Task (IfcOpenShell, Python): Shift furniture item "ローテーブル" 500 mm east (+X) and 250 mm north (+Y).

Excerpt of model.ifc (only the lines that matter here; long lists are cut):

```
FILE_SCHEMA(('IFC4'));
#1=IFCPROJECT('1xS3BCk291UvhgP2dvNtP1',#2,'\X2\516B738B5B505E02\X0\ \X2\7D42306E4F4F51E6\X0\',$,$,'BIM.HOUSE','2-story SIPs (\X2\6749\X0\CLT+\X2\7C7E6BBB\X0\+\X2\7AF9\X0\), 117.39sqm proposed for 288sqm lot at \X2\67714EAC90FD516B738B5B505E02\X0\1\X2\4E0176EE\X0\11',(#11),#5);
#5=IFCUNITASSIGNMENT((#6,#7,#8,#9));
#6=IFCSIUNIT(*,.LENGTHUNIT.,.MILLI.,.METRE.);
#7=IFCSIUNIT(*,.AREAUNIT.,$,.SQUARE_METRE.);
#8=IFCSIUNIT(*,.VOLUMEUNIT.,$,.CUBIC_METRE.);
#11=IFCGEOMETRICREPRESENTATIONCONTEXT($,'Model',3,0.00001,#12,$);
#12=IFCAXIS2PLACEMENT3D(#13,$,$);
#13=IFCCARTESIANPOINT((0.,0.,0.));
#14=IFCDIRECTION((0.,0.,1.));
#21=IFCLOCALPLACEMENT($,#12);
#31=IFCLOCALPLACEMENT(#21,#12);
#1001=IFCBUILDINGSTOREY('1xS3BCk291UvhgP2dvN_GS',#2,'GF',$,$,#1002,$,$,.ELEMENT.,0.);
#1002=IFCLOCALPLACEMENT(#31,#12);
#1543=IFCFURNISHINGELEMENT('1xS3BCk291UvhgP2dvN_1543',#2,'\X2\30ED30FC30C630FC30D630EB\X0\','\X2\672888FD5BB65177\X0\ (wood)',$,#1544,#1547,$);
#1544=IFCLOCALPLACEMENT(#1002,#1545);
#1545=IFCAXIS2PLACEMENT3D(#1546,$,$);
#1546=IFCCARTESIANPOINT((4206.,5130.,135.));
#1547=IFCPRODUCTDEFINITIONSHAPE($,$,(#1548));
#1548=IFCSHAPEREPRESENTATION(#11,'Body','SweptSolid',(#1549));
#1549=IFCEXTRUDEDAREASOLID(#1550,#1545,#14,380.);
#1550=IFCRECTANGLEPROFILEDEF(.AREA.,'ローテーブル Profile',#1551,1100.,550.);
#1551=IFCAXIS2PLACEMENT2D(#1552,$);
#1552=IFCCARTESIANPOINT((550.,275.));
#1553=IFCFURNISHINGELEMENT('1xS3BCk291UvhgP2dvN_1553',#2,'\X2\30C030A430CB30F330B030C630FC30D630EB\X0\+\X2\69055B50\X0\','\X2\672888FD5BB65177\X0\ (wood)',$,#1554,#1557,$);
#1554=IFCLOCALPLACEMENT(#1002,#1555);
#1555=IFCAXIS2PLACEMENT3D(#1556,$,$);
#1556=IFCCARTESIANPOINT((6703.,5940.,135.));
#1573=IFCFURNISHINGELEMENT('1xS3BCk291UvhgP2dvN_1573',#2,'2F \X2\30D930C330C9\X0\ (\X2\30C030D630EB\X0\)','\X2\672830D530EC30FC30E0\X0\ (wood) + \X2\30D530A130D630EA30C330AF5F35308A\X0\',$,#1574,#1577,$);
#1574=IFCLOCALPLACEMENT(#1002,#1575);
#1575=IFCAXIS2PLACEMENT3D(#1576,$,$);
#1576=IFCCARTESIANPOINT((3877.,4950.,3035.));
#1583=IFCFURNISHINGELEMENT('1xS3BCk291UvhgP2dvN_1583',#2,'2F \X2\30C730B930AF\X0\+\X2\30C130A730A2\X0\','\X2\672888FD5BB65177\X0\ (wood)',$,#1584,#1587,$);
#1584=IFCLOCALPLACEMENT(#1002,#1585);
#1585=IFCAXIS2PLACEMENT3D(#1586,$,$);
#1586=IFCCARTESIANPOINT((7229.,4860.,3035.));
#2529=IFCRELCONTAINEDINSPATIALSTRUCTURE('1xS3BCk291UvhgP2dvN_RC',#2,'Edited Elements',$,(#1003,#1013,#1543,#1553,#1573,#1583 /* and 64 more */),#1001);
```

```python
import ifcopenshell
import ifcopenshell.api.geometry
import ifcopenshell.util.placement
import ifcopenshell.util.unit

model = ifcopenshell.open("model.ifc")
unit_scale = ifcopenshell.util.unit.calculate_unit_scale(model)

item = model.by_guid("1xS3BCk291UvhgP2dvN_1543")
matrix = ifcopenshell.util.placement.get_local_placement(item.ObjectPlacement)
matrix[0, 3] += 0.5 / unit_scale
matrix[1, 3] += 0.25 / unit_scale
ifcopenshell.api.geometry.edit_object_placement(model, product=item, matrix=matrix, is_si=False)

print(ifcopenshell.util.placement.get_local_placement(item.ObjectPlacement).round(3) + 0.0)

model.write("model_updated.ifc")
```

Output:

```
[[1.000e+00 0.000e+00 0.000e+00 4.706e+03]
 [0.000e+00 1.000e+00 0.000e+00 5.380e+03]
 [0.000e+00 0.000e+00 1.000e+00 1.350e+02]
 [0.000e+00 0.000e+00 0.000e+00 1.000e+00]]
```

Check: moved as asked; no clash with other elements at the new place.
